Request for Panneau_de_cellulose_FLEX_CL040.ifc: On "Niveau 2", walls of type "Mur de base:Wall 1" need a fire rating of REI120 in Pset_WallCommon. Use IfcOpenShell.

First a look at what the model holds.

```python
import ifcopenshell
import ifcopenshell.util.element

model = ifcopenshell.open("Panneau_de_cellulose_FLEX_CL040.ifc")
print(model.schema)
storey = next(s for s in model.by_type("IfcBuildingStorey") if s.Name == "Niveau 2")
walls = [e for e in ifcopenshell.util.element.get_decomposition(storey) if e.is_a("IfcWall")]
seen = {}
for e in walls:
    element_type = ifcopenshell.util.element.get_type(e)
    key = (element_type.Name if element_type != e and element_type else None, ifcopenshell.util.element.get_pset(e, "Pset_WallCommon", "FireRating"))
    seen[key] = seen.get(key, 0) + 1
for (name, value), count in sorted(seen.items(), key=str):
    print(count, "x", name, "|", value)
```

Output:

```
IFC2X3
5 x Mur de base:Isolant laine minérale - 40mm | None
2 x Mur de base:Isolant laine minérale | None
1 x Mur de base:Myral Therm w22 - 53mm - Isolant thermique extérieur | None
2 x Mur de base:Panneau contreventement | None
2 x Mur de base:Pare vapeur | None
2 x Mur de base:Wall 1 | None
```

```python
import ifcopenshell
import ifcopenshell.api.pset
import ifcopenshell.util.element

model = ifcopenshell.open("Panneau_de_cellulose_FLEX_CL040.ifc")

storey = next(s for s in model.by_type("IfcBuildingStorey") if s.Name == "Niveau 2")
walls = [e for e in ifcopenshell.util.element.get_decomposition(storey) if e.is_a("IfcWall")]

count = 0
for e in walls:
    element_type = ifcopenshell.util.element.get_type(e)
    if element_type in (None, e) or element_type.Name != "Mur de base:Wall 1":
        continue
    # add_pset returns the element's existing set when there is one.
    pset = ifcopenshell.api.pset.add_pset(model, product=e, name="Pset_WallCommon")
    ifcopenshell.api.pset.edit_pset(model, pset=pset, properties={"FireRating": "REI120"})
    count += 1

print(count, "walls updated")

model.write("Panneau_de_cellulose_FLEX_CL040_updated.ifc")
```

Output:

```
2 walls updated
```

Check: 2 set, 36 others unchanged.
